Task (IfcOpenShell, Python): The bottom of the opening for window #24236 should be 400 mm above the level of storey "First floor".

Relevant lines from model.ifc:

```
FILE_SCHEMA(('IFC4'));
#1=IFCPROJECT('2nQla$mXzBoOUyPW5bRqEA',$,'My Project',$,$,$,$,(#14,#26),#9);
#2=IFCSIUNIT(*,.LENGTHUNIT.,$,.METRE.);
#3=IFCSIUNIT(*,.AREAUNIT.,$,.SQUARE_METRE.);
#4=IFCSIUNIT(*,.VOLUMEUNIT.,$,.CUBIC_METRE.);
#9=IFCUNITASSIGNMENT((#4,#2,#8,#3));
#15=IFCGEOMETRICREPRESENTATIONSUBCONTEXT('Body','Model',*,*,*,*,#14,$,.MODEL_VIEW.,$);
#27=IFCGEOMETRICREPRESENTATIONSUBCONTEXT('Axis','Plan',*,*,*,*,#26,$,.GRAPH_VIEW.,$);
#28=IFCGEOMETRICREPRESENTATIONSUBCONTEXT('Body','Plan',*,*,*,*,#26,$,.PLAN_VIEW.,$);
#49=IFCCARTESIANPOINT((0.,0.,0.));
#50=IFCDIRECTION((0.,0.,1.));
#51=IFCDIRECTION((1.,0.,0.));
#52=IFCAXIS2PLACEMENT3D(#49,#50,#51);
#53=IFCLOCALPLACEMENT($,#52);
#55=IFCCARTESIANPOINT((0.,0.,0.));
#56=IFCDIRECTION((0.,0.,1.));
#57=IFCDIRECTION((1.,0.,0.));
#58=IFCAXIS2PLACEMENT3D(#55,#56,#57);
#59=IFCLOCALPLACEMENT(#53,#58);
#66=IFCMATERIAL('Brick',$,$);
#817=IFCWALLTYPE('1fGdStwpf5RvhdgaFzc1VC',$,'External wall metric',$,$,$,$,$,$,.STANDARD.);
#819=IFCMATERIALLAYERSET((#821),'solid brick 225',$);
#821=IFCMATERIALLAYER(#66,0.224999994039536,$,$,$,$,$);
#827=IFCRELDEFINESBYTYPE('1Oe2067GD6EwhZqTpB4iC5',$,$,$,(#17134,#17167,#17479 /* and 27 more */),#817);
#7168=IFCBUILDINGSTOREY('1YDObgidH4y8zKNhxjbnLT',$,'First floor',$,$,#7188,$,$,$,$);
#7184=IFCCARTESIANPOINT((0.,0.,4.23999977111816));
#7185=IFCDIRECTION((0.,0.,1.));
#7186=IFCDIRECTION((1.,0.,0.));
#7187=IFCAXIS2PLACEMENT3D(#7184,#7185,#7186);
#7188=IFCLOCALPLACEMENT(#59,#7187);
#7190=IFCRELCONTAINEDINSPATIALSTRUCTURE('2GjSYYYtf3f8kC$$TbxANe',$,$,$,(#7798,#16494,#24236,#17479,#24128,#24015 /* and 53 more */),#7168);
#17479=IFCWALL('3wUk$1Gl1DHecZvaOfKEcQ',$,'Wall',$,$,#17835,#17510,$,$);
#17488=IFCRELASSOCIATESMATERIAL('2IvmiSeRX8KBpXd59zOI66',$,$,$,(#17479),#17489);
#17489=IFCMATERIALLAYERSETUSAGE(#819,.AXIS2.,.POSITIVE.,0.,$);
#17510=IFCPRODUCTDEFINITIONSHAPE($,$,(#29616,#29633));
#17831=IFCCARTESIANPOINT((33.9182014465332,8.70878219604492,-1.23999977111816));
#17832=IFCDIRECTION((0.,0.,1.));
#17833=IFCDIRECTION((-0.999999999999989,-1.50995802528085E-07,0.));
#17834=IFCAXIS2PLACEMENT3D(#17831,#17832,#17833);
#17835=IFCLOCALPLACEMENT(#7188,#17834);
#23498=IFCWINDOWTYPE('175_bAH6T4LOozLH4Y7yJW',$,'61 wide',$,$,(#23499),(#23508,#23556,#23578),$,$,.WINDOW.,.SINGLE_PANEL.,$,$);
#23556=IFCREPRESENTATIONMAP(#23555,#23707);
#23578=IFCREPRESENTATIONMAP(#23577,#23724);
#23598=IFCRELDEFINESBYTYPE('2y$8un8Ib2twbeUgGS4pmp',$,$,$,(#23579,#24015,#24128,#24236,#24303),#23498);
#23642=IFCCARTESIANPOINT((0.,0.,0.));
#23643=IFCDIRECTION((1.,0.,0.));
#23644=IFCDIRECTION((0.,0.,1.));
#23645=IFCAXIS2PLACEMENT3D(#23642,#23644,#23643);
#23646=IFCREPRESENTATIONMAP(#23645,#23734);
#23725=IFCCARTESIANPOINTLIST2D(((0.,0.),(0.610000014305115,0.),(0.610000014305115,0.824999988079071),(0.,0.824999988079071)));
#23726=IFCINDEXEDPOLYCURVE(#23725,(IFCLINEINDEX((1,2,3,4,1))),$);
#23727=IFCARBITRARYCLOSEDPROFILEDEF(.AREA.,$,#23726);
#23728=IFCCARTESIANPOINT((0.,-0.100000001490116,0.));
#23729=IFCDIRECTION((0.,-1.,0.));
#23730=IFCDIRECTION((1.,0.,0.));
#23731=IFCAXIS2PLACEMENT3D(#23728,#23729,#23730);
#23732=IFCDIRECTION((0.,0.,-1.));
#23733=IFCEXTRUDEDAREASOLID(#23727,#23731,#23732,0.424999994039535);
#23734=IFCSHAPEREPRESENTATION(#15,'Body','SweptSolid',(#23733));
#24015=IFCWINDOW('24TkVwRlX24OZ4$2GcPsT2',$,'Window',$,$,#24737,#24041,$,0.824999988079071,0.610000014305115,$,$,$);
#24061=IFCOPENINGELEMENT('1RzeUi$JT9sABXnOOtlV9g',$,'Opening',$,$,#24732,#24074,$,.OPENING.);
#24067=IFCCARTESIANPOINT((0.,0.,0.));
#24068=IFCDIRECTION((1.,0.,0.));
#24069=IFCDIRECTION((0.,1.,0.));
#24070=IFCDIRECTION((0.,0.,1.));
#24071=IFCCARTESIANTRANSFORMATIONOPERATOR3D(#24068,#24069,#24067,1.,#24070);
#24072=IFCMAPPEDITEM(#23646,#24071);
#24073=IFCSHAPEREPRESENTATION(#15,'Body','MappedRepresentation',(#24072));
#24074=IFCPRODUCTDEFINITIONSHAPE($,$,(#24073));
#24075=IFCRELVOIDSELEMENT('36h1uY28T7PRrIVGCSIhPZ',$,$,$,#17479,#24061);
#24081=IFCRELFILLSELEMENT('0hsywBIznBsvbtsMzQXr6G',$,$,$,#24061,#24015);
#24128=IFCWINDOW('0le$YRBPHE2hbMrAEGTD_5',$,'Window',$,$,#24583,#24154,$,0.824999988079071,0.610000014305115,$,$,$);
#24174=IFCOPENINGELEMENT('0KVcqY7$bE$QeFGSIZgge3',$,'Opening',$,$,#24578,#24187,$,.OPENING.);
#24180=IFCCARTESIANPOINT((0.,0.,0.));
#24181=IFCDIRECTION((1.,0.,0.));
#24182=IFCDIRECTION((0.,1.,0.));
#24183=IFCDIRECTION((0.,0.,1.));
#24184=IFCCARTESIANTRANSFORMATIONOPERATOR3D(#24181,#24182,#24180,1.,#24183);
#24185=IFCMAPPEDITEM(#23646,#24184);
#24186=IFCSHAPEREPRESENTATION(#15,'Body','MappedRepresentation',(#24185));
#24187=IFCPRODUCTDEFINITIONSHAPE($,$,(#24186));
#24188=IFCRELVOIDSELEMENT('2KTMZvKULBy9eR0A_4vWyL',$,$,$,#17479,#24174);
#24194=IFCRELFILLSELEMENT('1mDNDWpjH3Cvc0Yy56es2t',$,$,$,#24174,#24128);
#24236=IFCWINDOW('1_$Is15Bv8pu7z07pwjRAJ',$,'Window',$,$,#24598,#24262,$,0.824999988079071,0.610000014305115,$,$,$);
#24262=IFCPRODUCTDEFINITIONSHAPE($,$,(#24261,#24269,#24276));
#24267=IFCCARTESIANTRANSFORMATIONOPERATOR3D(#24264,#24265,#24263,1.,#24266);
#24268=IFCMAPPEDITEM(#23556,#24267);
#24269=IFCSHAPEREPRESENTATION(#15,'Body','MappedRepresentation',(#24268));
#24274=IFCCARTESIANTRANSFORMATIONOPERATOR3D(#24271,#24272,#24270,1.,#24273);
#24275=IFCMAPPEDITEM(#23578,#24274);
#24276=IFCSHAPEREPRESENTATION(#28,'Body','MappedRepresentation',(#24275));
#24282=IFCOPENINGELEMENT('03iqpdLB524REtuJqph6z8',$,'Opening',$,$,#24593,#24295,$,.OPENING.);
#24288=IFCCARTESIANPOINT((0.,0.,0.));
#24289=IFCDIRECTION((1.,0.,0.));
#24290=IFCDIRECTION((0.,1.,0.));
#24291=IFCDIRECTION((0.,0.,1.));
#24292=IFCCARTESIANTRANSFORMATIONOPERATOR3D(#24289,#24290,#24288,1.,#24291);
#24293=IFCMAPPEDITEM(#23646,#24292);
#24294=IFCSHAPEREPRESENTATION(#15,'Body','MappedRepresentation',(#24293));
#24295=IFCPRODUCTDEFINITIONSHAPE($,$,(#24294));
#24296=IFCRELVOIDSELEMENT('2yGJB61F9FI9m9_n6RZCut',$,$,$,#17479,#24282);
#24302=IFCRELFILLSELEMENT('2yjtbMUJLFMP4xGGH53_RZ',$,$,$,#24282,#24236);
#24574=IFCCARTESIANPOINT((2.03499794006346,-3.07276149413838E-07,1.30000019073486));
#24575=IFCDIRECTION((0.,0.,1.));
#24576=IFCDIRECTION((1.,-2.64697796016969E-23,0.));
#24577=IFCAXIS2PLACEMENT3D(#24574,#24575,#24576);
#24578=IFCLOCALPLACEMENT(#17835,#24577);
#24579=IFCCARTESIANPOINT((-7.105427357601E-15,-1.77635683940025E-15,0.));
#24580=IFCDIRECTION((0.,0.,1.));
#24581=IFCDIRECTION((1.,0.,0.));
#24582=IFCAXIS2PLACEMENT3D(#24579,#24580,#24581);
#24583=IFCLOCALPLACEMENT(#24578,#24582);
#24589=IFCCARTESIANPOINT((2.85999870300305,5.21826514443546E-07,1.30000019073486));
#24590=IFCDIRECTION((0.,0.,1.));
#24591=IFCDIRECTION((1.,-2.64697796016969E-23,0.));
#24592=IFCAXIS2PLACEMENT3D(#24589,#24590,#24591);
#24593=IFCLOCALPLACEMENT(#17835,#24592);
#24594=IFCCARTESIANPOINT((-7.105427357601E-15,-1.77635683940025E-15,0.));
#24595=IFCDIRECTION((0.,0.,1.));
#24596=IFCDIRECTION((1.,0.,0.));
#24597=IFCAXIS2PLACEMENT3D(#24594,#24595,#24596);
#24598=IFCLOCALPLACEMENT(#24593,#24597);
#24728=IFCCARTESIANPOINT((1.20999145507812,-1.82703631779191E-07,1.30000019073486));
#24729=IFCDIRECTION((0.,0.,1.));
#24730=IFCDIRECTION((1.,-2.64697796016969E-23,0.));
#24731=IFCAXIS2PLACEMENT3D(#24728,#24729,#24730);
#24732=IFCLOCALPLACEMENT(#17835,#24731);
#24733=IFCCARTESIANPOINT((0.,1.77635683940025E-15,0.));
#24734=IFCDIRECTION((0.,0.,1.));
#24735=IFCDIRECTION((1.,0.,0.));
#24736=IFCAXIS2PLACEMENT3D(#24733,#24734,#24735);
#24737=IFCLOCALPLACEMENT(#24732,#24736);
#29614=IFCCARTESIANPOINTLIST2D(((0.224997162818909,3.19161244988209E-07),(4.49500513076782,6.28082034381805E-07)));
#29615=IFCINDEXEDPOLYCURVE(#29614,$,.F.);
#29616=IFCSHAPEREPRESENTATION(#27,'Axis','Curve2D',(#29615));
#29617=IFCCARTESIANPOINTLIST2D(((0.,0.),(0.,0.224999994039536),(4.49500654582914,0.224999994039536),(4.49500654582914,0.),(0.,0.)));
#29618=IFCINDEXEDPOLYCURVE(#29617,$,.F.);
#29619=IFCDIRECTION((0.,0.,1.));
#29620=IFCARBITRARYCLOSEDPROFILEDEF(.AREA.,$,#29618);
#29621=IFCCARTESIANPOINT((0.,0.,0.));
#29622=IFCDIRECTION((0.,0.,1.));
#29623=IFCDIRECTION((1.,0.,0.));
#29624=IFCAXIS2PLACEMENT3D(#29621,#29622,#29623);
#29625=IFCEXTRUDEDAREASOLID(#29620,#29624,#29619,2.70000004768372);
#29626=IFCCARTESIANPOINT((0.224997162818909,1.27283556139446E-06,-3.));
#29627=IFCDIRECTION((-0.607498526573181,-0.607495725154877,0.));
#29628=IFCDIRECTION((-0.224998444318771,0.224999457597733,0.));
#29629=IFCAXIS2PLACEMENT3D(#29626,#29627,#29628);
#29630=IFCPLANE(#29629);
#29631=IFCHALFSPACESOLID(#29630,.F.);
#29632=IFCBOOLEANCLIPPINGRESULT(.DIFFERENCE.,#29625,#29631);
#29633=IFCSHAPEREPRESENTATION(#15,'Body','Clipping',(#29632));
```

```python
import numpy as np
import ifcopenshell
import ifcopenshell.api.geometry
import ifcopenshell.geom
import ifcopenshell.util.element
import ifcopenshell.util.placement
import ifcopenshell.util.shape
import ifcopenshell.util.unit

model = ifcopenshell.open("model.ifc")
unit_scale = ifcopenshell.util.unit.calculate_unit_scale(model)

window = model.by_guid("1_$Is15Bv8pu7z07pwjRAJ")
opening = window.FillsVoids[0].RelatingOpeningElement
storey = ifcopenshell.util.element.get_container(window, ifc_class="IfcBuildingStorey")
level = ifcopenshell.util.placement.get_local_placement(storey.ObjectPlacement)[2, 3]

# The opening's origin need not be at the sill, so measure its lowest point.
shape = ifcopenshell.geom.create_shape(ifcopenshell.geom.settings(), opening)
bottom = ifcopenshell.util.shape.get_shape_bottom_elevation(shape, shape.geometry) / unit_scale
dz = level + 0.4 / unit_scale - bottom

shift = np.array([0.0, 0.0, dz])
# The window is placed relative to its opening, so it follows when the opening moves.
matrix = ifcopenshell.util.placement.get_local_placement(opening.ObjectPlacement)
matrix[:3, 3] += shift
ifcopenshell.api.geometry.edit_object_placement(
    model, product=opening, matrix=matrix, is_si=False, should_transform_children=True
)

print(f"moved by {dz * unit_scale:+.3f} m")

model.write("model_edited.ifc")
```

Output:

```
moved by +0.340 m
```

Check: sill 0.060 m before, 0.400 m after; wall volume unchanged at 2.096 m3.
